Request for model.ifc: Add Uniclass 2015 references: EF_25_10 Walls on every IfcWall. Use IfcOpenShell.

First a look at what the model holds.

```python
import ifcopenshell

model = ifcopenshell.open("model.ifc")
print(model.schema)
print("classifications:", [c.Name for c in model.by_type("IfcClassification")])
for ifc_class in ("IfcDoor", "IfcRoof", "IfcStair", "IfcWall", "IfcWindow"):
    print(ifc_class, len(model.by_type(ifc_class)))
```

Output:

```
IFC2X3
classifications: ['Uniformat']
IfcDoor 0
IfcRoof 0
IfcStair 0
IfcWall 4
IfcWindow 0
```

```python
import ifcopenshell
import ifcopenshell.api.classification

model = ifcopenshell.open("model.ifc")

# IFC2X3 requires Source and Edition and has no link from the project to the system.
system = model.create_entity("IfcClassification", Source="NBS", Edition="2015", Name="Uniclass 2015")

codes = {
    "IfcWall": ("EF_25_10", "Walls"),
}
for ifc_class, (code, name) in codes.items():
    products = model.by_type(ifc_class)
    ifcopenshell.api.classification.add_reference(
        model, products=products, classification=system, identification=code, name=name
    )
    print(code, len(products))

model.write("model_updated.ifc")
```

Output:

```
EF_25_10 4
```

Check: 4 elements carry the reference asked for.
